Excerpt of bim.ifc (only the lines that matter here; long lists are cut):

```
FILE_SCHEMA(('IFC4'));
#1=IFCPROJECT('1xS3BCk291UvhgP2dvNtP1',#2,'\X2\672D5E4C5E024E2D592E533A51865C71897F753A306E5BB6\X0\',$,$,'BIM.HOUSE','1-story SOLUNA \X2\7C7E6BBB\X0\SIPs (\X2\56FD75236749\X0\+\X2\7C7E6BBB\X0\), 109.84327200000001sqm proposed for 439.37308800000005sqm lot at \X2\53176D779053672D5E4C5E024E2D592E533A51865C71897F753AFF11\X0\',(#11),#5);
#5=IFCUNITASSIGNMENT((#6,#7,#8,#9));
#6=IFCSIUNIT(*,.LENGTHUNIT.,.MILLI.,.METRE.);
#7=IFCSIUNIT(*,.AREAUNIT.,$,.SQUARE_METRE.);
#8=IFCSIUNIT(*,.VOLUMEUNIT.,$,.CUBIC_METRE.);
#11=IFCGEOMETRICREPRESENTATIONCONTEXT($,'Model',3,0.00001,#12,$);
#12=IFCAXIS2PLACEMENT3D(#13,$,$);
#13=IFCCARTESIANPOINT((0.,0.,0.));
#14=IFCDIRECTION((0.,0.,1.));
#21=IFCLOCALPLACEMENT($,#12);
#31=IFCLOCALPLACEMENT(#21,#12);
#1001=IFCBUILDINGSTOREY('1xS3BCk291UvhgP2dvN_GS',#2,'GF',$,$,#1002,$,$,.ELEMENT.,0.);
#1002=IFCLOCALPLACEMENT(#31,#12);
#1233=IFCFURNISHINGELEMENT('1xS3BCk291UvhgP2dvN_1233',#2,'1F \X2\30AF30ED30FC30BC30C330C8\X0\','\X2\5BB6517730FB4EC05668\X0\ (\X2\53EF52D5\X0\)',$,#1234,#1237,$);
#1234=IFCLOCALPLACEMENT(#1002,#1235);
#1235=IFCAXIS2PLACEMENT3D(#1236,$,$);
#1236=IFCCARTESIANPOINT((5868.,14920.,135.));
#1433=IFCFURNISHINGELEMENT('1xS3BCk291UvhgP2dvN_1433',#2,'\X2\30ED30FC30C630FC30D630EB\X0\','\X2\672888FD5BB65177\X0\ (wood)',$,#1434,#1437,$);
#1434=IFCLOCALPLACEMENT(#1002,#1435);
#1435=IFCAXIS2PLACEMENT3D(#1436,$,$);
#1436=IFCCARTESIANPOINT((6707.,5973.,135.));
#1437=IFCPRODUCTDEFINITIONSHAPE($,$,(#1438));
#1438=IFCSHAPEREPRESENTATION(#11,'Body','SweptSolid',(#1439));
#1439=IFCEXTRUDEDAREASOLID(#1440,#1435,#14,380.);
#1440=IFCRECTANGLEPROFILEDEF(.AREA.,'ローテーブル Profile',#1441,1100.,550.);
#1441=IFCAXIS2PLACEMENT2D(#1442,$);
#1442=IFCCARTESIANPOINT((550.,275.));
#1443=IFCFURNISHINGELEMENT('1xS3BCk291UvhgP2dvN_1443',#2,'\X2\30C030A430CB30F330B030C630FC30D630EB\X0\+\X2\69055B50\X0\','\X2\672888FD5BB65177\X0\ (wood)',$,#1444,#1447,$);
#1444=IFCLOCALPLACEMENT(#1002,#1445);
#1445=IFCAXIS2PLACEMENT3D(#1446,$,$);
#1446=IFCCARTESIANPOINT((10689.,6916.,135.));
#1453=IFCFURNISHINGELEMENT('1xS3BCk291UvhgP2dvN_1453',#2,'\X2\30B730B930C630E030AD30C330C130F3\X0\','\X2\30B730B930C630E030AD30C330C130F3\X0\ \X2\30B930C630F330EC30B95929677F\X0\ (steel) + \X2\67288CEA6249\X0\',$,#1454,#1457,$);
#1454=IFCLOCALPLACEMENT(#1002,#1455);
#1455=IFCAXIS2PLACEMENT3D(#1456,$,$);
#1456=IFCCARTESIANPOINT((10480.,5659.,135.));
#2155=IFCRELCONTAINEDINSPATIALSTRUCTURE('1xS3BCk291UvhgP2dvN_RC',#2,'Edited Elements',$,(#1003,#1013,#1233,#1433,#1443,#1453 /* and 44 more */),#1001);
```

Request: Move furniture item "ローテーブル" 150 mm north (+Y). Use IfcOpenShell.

```python
import ifcopenshell
import ifcopenshell.api.geometry
import ifcopenshell.util.placement
import ifcopenshell.util.unit

model = ifcopenshell.open("bim.ifc")
unit_scale = ifcopenshell.util.unit.calculate_unit_scale(model)

item = model.by_guid("1xS3BCk291UvhgP2dvN_1433")
matrix = ifcopenshell.util.placement.get_local_placement(item.ObjectPlacement)
matrix[1, 3] += 0.15 / unit_scale
ifcopenshell.api.geometry.edit_object_placement(model, product=item, matrix=matrix, is_si=False)

print(ifcopenshell.util.placement.get_local_placement(item.ObjectPlacement).round(3) + 0.0)

model.write("bim_rev.ifc")
```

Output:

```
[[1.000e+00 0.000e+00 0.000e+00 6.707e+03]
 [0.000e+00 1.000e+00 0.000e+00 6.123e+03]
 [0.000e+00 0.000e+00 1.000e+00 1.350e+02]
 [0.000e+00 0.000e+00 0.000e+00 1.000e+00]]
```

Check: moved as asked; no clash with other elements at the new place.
